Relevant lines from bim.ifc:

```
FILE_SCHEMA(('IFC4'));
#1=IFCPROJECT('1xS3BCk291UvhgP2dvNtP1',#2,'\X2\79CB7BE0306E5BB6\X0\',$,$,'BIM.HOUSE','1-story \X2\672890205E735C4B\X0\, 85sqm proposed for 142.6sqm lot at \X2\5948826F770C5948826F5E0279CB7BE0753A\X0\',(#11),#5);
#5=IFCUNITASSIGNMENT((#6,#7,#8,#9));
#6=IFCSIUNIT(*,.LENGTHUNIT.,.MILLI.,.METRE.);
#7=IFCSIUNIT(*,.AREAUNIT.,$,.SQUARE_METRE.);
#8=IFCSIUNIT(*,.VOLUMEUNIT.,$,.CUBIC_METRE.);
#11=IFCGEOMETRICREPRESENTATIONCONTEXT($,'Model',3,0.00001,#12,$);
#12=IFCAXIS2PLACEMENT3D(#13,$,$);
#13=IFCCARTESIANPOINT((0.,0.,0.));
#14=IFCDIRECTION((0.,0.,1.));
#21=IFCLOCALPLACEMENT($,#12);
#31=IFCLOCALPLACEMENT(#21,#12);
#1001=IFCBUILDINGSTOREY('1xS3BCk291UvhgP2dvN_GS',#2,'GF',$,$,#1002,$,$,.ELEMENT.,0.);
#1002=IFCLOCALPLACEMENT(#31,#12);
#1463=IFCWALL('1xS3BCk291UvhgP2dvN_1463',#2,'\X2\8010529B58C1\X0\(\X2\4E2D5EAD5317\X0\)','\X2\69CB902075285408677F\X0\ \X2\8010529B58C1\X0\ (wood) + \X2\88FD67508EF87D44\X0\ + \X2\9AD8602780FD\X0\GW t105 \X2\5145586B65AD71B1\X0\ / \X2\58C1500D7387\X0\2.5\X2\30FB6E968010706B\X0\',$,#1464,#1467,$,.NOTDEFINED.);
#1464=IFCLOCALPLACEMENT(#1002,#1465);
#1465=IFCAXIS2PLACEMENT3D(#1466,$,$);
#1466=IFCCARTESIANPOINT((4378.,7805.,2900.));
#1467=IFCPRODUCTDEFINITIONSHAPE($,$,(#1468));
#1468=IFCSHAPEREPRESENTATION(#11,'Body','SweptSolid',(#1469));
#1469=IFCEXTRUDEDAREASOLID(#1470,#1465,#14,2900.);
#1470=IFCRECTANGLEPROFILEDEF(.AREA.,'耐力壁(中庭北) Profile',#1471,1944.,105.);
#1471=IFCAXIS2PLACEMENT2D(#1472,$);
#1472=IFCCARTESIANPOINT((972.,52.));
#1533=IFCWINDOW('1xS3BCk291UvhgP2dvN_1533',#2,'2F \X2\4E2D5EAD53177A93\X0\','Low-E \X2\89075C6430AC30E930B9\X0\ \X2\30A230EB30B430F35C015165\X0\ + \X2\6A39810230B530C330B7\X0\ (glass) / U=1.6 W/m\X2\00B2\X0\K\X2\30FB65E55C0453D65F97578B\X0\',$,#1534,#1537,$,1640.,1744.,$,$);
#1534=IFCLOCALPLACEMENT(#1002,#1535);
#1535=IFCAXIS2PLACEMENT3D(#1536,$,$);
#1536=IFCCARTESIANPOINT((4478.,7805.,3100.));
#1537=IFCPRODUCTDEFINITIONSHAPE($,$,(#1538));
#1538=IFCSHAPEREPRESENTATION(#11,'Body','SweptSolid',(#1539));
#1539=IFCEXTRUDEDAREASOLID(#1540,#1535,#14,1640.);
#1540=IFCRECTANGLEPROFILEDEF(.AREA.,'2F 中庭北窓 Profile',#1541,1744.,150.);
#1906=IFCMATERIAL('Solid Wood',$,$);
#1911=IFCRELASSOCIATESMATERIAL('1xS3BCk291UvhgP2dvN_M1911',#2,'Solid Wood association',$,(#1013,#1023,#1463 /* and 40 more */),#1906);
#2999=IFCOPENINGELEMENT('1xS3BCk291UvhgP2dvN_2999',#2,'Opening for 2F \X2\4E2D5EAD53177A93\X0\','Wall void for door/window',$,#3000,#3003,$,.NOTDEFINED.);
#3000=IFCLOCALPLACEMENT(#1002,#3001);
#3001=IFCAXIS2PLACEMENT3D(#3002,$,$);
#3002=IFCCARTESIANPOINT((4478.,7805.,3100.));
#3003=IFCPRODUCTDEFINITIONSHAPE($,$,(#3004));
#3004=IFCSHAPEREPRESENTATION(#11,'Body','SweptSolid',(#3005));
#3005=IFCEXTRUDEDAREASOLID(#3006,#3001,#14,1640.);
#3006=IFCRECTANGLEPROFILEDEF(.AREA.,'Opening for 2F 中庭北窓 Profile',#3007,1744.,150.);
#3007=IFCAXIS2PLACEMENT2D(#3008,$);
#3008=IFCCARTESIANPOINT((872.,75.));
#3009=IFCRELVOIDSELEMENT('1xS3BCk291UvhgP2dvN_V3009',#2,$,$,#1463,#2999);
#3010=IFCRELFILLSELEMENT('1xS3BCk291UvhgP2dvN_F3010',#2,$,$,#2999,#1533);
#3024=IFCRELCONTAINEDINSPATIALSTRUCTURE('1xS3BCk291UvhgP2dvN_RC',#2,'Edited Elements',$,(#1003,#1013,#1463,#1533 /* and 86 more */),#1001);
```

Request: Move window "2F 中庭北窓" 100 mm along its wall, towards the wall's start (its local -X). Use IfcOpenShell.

```python
import ifcopenshell
import ifcopenshell.api.geometry
import ifcopenshell.util.placement
import ifcopenshell.util.unit

model = ifcopenshell.open("bim.ifc")
unit_scale = ifcopenshell.util.unit.calculate_unit_scale(model)

window = model.by_guid("1xS3BCk291UvhgP2dvN_1533")
opening = window.FillsVoids[0].RelatingOpeningElement
wall = opening.VoidsElements[0].RelatingBuildingElement

wall_matrix = ifcopenshell.util.placement.get_local_placement(wall.ObjectPlacement)
shift = wall_matrix[:3, 0] * -0.1 / unit_scale
before = ifcopenshell.util.placement.get_local_placement(window.ObjectPlacement)[:3, 3].copy()

# The window is not placed relative to its opening, so move both.
for product in (opening, window):
    matrix = ifcopenshell.util.placement.get_local_placement(product.ObjectPlacement)
    matrix[:3, 3] += shift
    ifcopenshell.api.geometry.edit_object_placement(model, product=product, matrix=matrix, is_si=False)

after = ifcopenshell.util.placement.get_local_placement(window.ObjectPlacement)[:3, 3]
print("window moved by", (after - before).round(3) + 0.0)

model.write("bim_updated.ifc")
```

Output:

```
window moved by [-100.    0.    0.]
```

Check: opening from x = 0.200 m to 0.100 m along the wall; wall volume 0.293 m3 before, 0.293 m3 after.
